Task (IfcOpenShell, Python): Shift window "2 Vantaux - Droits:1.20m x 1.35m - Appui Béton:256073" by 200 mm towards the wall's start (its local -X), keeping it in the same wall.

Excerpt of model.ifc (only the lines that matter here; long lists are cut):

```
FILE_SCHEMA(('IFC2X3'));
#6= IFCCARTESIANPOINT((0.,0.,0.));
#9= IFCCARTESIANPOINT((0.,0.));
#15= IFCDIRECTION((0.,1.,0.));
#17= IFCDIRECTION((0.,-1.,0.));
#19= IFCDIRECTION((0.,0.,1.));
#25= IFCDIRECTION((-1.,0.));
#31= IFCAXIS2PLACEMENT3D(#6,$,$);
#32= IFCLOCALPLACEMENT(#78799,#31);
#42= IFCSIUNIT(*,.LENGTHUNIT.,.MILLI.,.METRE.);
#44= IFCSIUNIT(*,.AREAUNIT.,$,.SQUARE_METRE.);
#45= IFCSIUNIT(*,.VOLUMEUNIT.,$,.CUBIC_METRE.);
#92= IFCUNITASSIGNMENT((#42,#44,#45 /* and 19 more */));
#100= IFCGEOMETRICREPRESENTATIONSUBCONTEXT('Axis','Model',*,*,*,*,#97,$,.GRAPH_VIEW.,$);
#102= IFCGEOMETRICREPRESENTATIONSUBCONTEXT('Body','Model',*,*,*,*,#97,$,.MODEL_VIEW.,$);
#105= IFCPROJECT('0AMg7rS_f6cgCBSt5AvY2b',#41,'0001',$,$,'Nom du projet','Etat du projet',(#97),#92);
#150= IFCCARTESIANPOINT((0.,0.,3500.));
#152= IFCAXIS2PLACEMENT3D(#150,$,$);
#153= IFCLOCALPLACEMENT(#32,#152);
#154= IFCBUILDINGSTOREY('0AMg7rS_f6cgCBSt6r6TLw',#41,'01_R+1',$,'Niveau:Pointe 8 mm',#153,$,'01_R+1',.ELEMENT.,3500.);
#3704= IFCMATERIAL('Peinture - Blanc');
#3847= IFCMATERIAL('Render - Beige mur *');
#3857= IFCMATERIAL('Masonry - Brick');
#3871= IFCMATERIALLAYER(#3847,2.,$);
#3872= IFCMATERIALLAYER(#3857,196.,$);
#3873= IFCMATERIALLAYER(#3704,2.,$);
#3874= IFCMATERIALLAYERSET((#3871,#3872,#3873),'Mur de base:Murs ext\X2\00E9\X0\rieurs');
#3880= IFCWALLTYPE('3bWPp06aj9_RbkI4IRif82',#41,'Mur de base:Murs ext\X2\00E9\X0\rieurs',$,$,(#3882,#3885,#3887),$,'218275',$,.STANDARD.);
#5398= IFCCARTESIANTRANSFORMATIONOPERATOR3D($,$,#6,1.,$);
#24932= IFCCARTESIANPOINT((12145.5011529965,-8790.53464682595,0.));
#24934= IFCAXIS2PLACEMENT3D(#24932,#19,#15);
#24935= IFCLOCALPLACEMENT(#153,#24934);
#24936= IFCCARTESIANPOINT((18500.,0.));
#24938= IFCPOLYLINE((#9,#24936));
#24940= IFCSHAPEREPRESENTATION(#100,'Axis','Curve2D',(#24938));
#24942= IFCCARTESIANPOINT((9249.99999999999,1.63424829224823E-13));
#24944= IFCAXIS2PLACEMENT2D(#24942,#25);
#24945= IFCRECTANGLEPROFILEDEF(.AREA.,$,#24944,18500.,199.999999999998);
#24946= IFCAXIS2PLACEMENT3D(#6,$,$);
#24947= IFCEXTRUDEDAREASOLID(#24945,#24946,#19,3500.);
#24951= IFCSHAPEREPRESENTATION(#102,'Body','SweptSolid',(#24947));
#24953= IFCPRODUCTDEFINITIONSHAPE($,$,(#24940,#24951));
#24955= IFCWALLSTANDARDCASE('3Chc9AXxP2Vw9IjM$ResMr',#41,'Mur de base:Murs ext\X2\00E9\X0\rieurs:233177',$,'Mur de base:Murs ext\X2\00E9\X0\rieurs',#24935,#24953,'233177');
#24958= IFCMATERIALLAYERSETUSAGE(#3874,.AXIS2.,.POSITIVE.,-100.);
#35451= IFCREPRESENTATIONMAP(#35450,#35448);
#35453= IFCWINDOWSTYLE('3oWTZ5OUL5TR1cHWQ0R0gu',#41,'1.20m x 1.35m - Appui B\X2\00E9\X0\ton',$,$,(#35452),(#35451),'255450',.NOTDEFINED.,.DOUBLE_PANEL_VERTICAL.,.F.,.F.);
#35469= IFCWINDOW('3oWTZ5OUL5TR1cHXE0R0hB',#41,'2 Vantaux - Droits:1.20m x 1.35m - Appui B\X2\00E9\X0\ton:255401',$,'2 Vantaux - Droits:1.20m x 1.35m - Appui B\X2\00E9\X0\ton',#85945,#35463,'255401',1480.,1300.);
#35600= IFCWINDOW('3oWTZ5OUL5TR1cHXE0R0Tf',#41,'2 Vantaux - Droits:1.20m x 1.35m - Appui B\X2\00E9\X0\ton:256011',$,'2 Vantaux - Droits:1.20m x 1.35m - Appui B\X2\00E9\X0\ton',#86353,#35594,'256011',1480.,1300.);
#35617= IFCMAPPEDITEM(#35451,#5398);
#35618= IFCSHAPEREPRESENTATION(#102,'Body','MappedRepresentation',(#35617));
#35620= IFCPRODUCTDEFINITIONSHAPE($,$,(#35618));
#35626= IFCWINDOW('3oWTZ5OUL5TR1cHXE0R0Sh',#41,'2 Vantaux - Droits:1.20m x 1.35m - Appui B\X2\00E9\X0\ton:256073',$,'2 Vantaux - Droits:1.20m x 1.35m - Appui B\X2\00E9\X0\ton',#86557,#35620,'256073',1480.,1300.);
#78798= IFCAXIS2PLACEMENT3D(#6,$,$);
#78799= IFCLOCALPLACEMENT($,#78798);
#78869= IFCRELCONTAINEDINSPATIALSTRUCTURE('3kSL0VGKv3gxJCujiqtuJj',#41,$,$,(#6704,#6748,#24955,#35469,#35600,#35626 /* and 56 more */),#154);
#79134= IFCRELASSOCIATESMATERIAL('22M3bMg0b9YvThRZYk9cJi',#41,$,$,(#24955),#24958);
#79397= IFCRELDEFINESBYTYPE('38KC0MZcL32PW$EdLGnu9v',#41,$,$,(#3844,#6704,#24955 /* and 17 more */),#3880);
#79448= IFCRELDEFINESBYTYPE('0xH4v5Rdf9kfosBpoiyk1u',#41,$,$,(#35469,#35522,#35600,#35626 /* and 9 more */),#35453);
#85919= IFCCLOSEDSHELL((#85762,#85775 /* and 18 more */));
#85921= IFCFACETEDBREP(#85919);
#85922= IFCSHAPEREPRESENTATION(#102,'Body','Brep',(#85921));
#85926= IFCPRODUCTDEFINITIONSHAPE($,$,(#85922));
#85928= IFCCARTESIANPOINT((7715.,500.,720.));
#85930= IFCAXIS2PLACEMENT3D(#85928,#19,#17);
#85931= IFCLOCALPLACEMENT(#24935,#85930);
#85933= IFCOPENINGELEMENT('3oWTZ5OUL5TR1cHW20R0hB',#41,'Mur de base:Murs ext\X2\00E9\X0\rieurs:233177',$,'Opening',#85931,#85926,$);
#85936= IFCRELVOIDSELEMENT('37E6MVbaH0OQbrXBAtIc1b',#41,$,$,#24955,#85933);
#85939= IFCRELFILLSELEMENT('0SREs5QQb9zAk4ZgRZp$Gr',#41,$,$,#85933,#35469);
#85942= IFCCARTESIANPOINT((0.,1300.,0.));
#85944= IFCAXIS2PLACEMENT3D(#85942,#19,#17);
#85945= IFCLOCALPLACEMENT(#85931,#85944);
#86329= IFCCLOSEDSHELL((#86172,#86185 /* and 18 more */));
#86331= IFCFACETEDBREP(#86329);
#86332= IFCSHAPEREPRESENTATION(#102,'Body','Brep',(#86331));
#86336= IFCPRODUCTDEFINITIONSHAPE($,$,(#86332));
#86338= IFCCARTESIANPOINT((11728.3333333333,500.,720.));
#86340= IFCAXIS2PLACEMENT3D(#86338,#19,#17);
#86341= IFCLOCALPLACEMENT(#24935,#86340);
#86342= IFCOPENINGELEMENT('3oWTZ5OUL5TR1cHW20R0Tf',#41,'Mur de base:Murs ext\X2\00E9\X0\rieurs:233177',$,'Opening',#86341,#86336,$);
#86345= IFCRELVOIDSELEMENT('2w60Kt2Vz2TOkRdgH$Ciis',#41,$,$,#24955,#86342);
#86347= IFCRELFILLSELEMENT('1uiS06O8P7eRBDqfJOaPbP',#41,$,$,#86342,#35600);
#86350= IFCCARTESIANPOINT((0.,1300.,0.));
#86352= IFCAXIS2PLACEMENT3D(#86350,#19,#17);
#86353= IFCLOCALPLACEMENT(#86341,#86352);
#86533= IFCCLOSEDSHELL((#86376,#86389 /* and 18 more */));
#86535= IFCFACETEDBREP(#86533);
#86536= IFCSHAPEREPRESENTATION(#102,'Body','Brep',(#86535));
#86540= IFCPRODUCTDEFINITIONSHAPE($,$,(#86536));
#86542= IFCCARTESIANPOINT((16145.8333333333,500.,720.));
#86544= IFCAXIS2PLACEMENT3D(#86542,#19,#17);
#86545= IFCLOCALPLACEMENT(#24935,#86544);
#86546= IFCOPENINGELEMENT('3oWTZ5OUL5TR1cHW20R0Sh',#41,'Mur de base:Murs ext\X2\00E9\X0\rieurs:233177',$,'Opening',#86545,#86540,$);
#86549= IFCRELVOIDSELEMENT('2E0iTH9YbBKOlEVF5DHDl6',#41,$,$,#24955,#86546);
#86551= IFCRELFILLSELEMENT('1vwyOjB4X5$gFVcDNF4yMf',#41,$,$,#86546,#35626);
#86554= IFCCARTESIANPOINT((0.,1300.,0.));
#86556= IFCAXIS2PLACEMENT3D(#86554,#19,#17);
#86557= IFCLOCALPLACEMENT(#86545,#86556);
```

```python
import ifcopenshell
import ifcopenshell.api.geometry
import ifcopenshell.util.placement
import ifcopenshell.util.unit

model = ifcopenshell.open("model.ifc")
unit_scale = ifcopenshell.util.unit.calculate_unit_scale(model)

window = model.by_guid("3oWTZ5OUL5TR1cHXE0R0Sh")
opening = window.FillsVoids[0].RelatingOpeningElement
wall = opening.VoidsElements[0].RelatingBuildingElement

wall_matrix = ifcopenshell.util.placement.get_local_placement(wall.ObjectPlacement)
shift = wall_matrix[:3, 0] * -0.2 / unit_scale
before = ifcopenshell.util.placement.get_local_placement(window.ObjectPlacement)[:3, 3].copy()

# The window is placed relative to its opening, so it follows when the opening moves.
matrix = ifcopenshell.util.placement.get_local_placement(opening.ObjectPlacement)
matrix[:3, 3] += shift
ifcopenshell.api.geometry.edit_object_placement(
    model, product=opening, matrix=matrix, is_si=False, should_transform_children=True
)

after = ifcopenshell.util.placement.get_local_placement(window.ObjectPlacement)[:3, 3]
print("window moved by", (after - before).round(3) + 0.0)

model.write("model-out.ifc")
```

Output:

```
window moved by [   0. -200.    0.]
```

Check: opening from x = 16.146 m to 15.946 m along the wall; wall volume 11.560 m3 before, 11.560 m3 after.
